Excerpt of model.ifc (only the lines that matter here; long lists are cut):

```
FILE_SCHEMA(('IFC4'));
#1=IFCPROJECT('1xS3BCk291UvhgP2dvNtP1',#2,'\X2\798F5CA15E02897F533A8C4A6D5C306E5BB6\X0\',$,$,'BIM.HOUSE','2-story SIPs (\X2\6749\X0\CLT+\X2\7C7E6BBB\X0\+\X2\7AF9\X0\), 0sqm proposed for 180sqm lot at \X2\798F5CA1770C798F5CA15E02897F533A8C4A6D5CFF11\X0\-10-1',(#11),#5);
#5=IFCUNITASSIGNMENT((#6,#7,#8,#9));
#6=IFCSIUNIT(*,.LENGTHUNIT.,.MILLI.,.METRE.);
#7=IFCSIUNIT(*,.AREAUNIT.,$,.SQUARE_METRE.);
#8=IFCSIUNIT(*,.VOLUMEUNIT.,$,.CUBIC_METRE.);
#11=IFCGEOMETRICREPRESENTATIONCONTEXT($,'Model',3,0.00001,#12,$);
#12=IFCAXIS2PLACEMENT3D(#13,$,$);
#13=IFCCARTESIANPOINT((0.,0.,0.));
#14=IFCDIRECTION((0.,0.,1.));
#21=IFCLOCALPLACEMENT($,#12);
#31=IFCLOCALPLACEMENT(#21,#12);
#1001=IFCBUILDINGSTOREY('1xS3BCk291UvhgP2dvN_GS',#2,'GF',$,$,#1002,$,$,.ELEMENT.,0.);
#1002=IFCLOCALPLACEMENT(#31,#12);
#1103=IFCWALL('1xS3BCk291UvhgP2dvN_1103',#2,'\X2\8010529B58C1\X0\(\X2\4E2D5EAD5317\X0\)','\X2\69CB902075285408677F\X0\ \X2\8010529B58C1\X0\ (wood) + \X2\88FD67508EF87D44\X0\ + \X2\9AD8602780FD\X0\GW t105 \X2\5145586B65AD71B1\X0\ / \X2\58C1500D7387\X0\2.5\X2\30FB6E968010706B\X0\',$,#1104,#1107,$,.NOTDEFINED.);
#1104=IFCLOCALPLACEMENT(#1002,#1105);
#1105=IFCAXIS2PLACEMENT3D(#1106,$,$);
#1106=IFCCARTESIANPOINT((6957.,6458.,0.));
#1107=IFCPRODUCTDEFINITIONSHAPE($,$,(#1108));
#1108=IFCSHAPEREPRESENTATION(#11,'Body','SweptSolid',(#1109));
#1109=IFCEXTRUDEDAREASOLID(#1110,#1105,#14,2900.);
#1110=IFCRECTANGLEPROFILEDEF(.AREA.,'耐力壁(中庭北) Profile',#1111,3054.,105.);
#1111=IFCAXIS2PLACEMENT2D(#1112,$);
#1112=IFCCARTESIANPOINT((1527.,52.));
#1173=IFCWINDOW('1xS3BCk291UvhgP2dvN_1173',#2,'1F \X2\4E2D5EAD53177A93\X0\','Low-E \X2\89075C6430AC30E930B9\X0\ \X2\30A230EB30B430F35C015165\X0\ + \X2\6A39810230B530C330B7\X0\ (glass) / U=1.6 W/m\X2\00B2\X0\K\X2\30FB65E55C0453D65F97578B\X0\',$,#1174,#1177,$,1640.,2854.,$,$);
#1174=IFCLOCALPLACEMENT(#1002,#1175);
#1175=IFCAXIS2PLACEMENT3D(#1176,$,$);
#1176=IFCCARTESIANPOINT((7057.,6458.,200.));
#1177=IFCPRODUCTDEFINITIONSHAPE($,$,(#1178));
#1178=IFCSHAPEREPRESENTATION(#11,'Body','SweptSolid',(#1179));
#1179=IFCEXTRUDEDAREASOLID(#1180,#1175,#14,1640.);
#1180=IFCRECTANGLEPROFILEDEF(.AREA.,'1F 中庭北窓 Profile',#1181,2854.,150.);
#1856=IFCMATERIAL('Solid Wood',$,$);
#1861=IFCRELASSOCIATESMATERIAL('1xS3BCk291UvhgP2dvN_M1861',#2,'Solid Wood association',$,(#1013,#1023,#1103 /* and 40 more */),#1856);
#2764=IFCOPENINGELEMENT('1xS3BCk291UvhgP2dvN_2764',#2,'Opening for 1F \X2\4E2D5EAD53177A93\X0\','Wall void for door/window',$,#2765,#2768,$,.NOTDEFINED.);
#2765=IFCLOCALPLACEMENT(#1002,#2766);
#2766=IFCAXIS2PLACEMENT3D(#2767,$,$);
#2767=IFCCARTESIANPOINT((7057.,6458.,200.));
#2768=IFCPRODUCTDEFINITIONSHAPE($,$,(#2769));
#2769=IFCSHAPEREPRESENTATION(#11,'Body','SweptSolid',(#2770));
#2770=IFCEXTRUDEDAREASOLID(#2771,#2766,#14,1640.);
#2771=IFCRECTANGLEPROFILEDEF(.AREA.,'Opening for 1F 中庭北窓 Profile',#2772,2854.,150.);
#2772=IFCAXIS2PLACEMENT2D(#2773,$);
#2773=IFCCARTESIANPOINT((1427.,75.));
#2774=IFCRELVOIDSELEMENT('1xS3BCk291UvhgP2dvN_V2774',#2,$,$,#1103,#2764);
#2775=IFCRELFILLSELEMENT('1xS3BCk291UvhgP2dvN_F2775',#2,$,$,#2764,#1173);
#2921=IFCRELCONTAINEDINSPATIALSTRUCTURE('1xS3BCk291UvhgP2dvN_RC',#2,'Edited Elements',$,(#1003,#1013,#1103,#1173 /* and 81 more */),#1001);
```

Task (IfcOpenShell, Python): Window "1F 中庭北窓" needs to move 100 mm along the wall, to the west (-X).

```python
import ifcopenshell
import ifcopenshell.api.geometry
import ifcopenshell.util.placement

model = ifcopenshell.open("model.ifc")

window = model.by_guid("1xS3BCk291UvhgP2dvN_1173")
opening = window.FillsVoids[0].RelatingOpeningElement
wall = opening.VoidsElements[0].RelatingBuildingElement

wall_matrix = ifcopenshell.util.placement.get_local_placement(wall.ObjectPlacement)
shift = wall_matrix[:3, 0] * -100.0
before = ifcopenshell.util.placement.get_local_placement(window.ObjectPlacement)[:3, 3].copy()

# The window is not placed relative to its opening, so move both.
for product in (opening, window):
    matrix = ifcopenshell.util.placement.get_local_placement(product.ObjectPlacement)
    matrix[:3, 3] += shift
    ifcopenshell.api.geometry.edit_object_placement(model, product=product, matrix=matrix, is_si=False)

after = ifcopenshell.util.placement.get_local_placement(window.ObjectPlacement)[:3, 3]
print("window moved by", (after - before).round(3) + 0.0)

model.write("model-out.ifc")
```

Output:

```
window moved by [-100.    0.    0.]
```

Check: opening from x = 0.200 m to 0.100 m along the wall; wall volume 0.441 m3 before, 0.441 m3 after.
